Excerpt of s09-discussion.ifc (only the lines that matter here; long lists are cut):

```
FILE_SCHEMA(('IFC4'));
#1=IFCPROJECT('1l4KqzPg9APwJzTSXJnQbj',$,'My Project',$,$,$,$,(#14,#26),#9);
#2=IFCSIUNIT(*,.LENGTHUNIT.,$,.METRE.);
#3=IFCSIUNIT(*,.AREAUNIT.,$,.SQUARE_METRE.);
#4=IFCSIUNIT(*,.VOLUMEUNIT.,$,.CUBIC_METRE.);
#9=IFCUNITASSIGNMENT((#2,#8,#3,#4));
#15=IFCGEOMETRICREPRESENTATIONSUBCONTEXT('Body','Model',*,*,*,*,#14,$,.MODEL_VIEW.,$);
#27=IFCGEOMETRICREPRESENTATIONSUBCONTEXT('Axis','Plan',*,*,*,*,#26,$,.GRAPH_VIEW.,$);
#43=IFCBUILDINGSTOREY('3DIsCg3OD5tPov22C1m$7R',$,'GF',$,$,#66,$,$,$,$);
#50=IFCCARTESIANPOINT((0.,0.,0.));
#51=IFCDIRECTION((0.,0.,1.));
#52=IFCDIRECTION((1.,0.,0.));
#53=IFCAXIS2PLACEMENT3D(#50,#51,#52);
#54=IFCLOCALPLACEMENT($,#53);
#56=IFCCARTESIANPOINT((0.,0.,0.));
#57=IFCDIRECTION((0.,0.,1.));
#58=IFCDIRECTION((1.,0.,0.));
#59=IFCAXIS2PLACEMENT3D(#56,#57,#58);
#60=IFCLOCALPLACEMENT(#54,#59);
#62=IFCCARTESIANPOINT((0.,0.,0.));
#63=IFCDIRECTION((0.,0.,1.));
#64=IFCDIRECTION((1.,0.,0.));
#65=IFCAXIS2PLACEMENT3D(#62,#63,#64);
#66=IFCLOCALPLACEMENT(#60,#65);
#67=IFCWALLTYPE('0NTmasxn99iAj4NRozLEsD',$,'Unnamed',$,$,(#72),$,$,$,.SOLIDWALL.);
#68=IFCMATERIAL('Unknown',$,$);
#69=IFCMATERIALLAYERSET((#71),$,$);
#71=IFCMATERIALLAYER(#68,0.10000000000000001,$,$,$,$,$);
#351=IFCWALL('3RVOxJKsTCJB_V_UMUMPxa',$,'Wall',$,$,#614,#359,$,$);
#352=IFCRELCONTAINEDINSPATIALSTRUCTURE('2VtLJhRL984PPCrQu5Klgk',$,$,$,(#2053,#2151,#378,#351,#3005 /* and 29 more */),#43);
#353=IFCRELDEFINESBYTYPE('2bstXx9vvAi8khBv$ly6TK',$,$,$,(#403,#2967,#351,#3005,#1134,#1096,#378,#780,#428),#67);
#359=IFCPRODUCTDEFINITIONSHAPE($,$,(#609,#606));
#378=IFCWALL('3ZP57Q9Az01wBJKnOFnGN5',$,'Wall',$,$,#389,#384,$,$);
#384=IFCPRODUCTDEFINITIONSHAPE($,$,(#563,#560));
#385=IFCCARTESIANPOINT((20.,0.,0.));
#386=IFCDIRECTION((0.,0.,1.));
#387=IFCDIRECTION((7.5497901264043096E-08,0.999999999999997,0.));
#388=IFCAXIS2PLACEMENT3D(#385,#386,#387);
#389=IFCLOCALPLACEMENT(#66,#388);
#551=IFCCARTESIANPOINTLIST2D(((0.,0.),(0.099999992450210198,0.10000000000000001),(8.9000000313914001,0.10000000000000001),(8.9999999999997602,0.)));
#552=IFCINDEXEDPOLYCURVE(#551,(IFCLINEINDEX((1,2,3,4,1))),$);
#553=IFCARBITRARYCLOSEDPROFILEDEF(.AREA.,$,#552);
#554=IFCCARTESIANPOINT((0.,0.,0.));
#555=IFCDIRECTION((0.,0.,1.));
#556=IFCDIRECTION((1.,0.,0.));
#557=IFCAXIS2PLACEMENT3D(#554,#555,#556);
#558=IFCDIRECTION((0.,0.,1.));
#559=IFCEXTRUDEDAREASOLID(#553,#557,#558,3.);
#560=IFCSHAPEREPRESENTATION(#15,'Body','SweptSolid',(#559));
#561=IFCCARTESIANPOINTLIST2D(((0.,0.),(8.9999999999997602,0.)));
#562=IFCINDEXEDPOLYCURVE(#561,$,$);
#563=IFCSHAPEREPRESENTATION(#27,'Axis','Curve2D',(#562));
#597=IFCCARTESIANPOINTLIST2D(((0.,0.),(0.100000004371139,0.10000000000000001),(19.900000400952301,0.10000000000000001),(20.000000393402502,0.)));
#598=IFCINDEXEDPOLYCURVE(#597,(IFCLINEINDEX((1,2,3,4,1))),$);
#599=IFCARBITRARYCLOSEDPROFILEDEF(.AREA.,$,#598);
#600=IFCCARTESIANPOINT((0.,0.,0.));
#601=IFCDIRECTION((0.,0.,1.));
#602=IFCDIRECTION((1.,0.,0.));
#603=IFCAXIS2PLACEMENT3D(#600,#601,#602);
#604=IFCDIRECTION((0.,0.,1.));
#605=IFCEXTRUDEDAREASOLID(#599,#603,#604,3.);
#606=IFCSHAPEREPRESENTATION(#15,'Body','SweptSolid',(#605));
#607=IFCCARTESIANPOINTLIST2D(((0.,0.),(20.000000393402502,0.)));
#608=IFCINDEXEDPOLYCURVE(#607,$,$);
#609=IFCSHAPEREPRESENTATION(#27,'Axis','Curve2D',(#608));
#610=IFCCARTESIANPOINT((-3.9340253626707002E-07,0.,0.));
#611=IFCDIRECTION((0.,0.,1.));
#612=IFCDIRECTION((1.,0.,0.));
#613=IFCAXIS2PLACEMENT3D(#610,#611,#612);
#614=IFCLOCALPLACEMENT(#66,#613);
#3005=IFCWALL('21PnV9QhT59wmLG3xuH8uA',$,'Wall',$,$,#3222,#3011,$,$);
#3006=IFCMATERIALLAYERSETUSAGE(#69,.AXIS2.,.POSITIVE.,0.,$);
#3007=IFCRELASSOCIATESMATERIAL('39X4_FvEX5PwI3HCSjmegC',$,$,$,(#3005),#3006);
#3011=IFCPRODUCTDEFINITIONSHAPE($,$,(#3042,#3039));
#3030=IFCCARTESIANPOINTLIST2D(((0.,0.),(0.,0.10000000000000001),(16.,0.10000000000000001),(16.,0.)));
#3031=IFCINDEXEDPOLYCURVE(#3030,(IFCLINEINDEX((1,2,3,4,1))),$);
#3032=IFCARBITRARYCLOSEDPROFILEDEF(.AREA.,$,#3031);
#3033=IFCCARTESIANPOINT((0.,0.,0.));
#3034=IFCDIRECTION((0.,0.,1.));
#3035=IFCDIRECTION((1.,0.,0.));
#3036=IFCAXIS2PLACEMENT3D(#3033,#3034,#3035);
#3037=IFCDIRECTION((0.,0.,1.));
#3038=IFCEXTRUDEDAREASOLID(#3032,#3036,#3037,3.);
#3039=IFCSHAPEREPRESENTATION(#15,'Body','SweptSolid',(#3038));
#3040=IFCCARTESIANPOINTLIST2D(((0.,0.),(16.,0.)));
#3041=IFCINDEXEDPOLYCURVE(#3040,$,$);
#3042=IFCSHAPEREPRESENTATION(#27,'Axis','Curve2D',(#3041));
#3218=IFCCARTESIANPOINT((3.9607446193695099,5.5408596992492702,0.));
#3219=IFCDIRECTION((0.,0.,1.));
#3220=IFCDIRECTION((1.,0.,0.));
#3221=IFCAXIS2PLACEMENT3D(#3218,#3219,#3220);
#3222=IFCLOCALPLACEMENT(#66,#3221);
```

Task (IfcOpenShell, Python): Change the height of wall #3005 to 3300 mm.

```python
import ifcopenshell
import ifcopenshell.geom
import ifcopenshell.util.representation
import ifcopenshell.util.shape
import ifcopenshell.util.unit

model = ifcopenshell.open("s09-discussion.ifc")
unit_scale = ifcopenshell.util.unit.calculate_unit_scale(model)
settings = ifcopenshell.geom.settings()


def volume(element):
    """Net volume in cubic metres, openings subtracted."""
    shape = ifcopenshell.geom.create_shape(settings, element)
    return ifcopenshell.util.shape.get_volume(shape.geometry)


wall = model.by_id(3005)
before = volume(wall)

body = ifcopenshell.util.representation.get_representation(wall, "Model", "Body")
solid = body.Items[0]
old_height = solid.Depth
solid.Depth = 3.3 / unit_scale
after = volume(wall)

print(f"height {old_height:g} -> {solid.Depth:g}, volume {before:.3f} -> {after:.3f} m3")

model.write("s09-discussion_updated.ifc")
```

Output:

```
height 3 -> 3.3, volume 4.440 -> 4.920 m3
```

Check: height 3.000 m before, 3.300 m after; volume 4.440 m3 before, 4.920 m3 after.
